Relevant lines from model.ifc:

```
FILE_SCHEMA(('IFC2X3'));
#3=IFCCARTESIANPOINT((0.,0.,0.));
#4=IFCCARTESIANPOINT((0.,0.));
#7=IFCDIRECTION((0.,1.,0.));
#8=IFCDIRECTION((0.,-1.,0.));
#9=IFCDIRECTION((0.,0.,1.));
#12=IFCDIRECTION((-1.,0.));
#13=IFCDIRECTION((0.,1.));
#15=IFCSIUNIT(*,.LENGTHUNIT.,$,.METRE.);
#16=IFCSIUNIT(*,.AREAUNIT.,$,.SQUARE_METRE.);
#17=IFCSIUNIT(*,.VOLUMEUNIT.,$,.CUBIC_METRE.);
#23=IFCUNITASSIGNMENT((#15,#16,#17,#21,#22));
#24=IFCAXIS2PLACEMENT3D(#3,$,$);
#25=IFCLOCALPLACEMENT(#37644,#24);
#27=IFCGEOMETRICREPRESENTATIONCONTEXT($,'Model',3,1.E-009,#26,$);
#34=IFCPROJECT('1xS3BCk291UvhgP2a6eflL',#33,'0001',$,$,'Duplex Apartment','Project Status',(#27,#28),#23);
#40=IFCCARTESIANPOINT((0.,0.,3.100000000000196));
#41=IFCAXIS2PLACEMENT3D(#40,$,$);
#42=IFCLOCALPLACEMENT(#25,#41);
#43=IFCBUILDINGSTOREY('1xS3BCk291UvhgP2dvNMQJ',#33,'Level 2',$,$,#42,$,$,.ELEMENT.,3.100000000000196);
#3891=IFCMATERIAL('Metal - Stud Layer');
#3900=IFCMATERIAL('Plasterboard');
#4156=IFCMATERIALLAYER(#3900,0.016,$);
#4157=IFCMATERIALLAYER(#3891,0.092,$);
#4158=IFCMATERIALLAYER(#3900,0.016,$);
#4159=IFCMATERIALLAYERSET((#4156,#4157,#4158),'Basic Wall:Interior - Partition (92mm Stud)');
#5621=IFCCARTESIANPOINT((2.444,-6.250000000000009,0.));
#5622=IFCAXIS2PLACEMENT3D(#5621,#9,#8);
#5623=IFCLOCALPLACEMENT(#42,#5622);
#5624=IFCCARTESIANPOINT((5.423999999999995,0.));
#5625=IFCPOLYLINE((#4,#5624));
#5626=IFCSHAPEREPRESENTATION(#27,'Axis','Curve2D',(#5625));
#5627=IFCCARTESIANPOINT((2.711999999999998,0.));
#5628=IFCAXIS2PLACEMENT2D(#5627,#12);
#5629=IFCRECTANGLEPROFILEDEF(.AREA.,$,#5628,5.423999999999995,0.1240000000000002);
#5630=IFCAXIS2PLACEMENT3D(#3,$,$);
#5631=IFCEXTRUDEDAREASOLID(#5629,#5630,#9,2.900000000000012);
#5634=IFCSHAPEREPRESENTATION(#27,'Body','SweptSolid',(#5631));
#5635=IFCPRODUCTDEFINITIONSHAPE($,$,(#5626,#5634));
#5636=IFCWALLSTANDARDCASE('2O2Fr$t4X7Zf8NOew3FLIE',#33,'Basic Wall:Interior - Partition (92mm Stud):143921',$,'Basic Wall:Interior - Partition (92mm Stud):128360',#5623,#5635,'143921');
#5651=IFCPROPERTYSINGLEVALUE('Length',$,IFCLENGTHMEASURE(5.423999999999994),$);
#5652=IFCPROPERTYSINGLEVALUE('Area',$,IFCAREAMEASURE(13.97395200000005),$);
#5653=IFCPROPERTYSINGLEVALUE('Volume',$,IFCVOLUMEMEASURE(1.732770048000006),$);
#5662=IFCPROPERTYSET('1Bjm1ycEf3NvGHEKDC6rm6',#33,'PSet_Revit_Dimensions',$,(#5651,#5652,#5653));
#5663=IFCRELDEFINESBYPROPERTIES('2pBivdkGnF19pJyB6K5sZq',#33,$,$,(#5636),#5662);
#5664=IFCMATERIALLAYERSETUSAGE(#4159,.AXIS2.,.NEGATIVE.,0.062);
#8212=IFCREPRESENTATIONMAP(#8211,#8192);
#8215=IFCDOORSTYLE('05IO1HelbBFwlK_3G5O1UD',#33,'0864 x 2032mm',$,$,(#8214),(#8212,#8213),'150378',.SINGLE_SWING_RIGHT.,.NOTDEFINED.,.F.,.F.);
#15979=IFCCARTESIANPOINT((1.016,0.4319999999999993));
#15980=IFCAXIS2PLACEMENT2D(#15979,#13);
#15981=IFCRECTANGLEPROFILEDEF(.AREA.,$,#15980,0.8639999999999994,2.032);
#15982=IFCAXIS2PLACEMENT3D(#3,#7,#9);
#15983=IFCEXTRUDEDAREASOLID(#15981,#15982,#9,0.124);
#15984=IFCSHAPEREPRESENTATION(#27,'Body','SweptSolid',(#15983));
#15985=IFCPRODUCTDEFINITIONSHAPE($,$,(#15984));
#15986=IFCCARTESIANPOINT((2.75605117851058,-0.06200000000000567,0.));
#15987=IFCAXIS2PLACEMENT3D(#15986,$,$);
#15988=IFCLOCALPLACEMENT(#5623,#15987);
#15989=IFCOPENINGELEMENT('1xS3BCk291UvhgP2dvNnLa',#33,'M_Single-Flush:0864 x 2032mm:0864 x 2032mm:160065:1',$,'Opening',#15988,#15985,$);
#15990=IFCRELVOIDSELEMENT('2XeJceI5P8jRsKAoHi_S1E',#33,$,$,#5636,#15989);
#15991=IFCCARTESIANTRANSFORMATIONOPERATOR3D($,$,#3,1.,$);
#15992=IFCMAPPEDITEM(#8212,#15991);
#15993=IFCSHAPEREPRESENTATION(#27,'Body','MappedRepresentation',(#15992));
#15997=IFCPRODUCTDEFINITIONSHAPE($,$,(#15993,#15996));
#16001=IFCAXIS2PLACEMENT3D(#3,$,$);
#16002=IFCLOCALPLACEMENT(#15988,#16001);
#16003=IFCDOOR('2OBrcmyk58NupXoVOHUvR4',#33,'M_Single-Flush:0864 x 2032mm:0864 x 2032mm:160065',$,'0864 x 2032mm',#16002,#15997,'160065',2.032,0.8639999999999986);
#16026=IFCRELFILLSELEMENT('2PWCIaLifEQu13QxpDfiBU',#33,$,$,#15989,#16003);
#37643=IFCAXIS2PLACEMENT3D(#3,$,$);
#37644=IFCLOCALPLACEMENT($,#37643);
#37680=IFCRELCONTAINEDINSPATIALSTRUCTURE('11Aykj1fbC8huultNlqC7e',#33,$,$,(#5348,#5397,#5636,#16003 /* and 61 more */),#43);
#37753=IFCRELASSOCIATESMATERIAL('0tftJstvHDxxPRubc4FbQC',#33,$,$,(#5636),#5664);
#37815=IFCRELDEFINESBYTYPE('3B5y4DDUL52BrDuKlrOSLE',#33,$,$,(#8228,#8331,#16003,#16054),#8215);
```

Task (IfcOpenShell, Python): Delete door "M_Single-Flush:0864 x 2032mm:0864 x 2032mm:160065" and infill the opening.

```python
import ifcopenshell
import ifcopenshell.api.feature
import ifcopenshell.api.pset
import ifcopenshell.api.root
import ifcopenshell.geom
import ifcopenshell.util.element
import ifcopenshell.util.shape
import ifcopenshell.util.unit

model = ifcopenshell.open("model.ifc")
area_scale = ifcopenshell.util.unit.calculate_unit_scale(model, "AREAUNIT")
volume_scale = ifcopenshell.util.unit.calculate_unit_scale(model, "VOLUMEUNIT")
settings = ifcopenshell.geom.settings()


def volume(element):
    """Net volume in cubic metres, openings subtracted."""
    shape = ifcopenshell.geom.create_shape(settings, element)
    return ifcopenshell.util.shape.get_volume(shape.geometry)


door = model.by_guid("2OBrcmyk58NupXoVOHUvR4")
opening = door.FillsVoids[0].RelatingOpeningElement
wall = opening.VoidsElements[0].RelatingBuildingElement
before = volume(wall)

ifcopenshell.api.root.remove_product(model, product=door)
ifcopenshell.api.feature.remove_feature(model, feature=opening)

after = volume(wall)
thickness = 0.124  # wall thickness in metres

# Update the wall's stored quantities.
pset = model.by_id(ifcopenshell.util.element.get_pset(wall, "PSet_Revit_Dimensions", should_inherit=False)["id"])
ifcopenshell.api.pset.edit_pset(model, pset=pset, properties={
    "Area": model.create_entity("IfcAreaMeasure", after / thickness / area_scale),
    "Volume": model.create_entity("IfcVolumeMeasure", after / volume_scale),
})

print(f"wall volume {before:.3f} -> {after:.3f} m3")

model.write("model_rev.ifc")
```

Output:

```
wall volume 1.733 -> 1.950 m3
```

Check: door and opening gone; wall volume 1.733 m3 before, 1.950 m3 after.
